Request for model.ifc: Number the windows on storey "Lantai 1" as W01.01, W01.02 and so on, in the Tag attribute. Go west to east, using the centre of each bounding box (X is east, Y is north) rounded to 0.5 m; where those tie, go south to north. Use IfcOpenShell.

First a look at what the model holds.

```python
import ifcopenshell
import ifcopenshell.util.element
import ifcopenshell.util.placement

model = ifcopenshell.open("model.ifc")
print(model.schema)
storey = next(s for s in model.by_type("IfcBuildingStorey") if s.Name == "Lantai 1")
windows = [e for e in ifcopenshell.util.element.get_decomposition(storey) if e.is_a("IfcWindow")]
for e in sorted(windows, key=lambda e: e.id()):
    origin = ifcopenshell.util.placement.get_local_placement(e.ObjectPlacement)[:3, 3]
    print(e.id(), e.Tag, e.Name, origin.round(2) + 0.0, sep=" | ")
```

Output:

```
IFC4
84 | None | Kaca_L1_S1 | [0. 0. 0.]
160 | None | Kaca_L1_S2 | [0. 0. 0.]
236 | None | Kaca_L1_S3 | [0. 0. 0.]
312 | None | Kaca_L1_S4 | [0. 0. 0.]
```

```python
import ifcopenshell
import ifcopenshell.geom
import ifcopenshell.util.element
import ifcopenshell.util.shape

model = ifcopenshell.open("model.ifc")
settings = ifcopenshell.geom.settings()
settings.set("use-world-coords", True)


def centre(element):
    shape = ifcopenshell.geom.create_shape(settings, element)
    return ifcopenshell.util.shape.get_bbox_centroid(shape.geometry)


storey = next(s for s in model.by_type("IfcBuildingStorey") if s.Name == "Lantai 1")
windows = [e for e in ifcopenshell.util.element.get_decomposition(storey) if e.is_a("IfcWindow")]

# Insertion points can sit at a corner or the storey origin, so sort by the geometry (in metres).
centres = {e: centre(e) for e in windows}
windows.sort(key=lambda e: (round(centres[e][0] / 0.5), centres[e][1]))

for i, e in enumerate(windows, start=1):
    number = f"W01.{i:02d}"
    e.Tag = number
    print(e.id(), number)

model.write("model_v2.ifc")
```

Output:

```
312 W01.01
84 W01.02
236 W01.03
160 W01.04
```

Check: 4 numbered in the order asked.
